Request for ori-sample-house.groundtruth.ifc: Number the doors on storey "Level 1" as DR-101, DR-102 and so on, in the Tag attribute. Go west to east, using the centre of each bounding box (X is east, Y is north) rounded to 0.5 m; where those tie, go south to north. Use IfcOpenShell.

First a look at what the model holds.

```python
import ifcopenshell
import ifcopenshell.util.element
import ifcopenshell.util.placement

model = ifcopenshell.open("ori-sample-house.groundtruth.ifc")
print(model.schema)
storey = next(s for s in model.by_type("IfcBuildingStorey") if s.Name == "Level 1")
doors = [e for e in ifcopenshell.util.element.get_decomposition(storey) if e.is_a("IfcDoor")]
for e in sorted(doors, key=lambda e: e.id()):
    origin = ifcopenshell.util.placement.get_local_placement(e.ObjectPlacement)[:3, 3]
    print(e.id(), e.Tag, e.Name, origin.round(2) + 0.0, sep=" | ")
```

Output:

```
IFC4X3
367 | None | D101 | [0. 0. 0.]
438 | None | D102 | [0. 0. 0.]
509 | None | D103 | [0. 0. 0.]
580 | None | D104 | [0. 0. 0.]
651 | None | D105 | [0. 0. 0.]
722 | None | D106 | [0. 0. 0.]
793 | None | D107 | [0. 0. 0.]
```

```python
import ifcopenshell
import ifcopenshell.geom
import ifcopenshell.util.element
import ifcopenshell.util.shape

model = ifcopenshell.open("ori-sample-house.groundtruth.ifc")
settings = ifcopenshell.geom.settings()
settings.set("use-world-coords", True)


def centre(element):
    shape = ifcopenshell.geom.create_shape(settings, element)
    return ifcopenshell.util.shape.get_bbox_centroid(shape.geometry)


storey = next(s for s in model.by_type("IfcBuildingStorey") if s.Name == "Level 1")
doors = [e for e in ifcopenshell.util.element.get_decomposition(storey) if e.is_a("IfcDoor")]

# Insertion points can sit at a corner or the storey origin, so sort by the geometry (in metres).
centres = {e: centre(e) for e in doors}
doors.sort(key=lambda e: (round(centres[e][0] / 0.5), centres[e][1]))

for i, e in enumerate(doors, start=1):
    number = f"DR-1{i:02d}"
    e.Tag = number
    print(e.id(), number)

model.write("ori-sample-house.groundtruth_rev.ifc")
```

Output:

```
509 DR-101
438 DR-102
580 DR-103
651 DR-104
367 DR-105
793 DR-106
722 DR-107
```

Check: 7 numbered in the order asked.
